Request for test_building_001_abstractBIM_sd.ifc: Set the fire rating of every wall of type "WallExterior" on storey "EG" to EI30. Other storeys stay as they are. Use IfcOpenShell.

First a look at what the model holds.

```python
import ifcopenshell
import ifcopenshell.util.element

model = ifcopenshell.open("test_building_001_abstractBIM_sd.ifc")
print(model.schema)
storey = next(s for s in model.by_type("IfcBuildingStorey") if s.Name == "EG")
walls = [e for e in ifcopenshell.util.element.get_decomposition(storey) if e.is_a("IfcWall")]
seen = {}
for e in walls:
    element_type = ifcopenshell.util.element.get_type(e)
    key = (element_type.Name if element_type != e and element_type else None, ifcopenshell.util.element.get_pset(e, "Pset_WallCommon", "FireRating"))
    seen[key] = seen.get(key, 0) + 1
for (name, value), count in sorted(seen.items(), key=str):
    print(count, "x", name, "|", value)
```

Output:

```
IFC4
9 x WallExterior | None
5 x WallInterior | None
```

```python
import ifcopenshell
import ifcopenshell.api.pset
import ifcopenshell.util.element

model = ifcopenshell.open("test_building_001_abstractBIM_sd.ifc")

storey = next(s for s in model.by_type("IfcBuildingStorey") if s.Name == "EG")
walls = [e for e in ifcopenshell.util.element.get_decomposition(storey) if e.is_a("IfcWall")]

count = 0
for e in walls:
    element_type = ifcopenshell.util.element.get_type(e)
    if element_type in (None, e) or element_type.Name != "WallExterior":
        continue
    # add_pset returns the element's existing set when there is one.
    pset = ifcopenshell.api.pset.add_pset(model, product=e, name="Pset_WallCommon")
    ifcopenshell.api.pset.edit_pset(model, pset=pset, properties={"FireRating": "EI30"})
    count += 1

print(count, "walls updated")

model.write("test_building_001_abstractBIM_sd_rev.ifc")
```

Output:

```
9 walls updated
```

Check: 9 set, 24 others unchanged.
